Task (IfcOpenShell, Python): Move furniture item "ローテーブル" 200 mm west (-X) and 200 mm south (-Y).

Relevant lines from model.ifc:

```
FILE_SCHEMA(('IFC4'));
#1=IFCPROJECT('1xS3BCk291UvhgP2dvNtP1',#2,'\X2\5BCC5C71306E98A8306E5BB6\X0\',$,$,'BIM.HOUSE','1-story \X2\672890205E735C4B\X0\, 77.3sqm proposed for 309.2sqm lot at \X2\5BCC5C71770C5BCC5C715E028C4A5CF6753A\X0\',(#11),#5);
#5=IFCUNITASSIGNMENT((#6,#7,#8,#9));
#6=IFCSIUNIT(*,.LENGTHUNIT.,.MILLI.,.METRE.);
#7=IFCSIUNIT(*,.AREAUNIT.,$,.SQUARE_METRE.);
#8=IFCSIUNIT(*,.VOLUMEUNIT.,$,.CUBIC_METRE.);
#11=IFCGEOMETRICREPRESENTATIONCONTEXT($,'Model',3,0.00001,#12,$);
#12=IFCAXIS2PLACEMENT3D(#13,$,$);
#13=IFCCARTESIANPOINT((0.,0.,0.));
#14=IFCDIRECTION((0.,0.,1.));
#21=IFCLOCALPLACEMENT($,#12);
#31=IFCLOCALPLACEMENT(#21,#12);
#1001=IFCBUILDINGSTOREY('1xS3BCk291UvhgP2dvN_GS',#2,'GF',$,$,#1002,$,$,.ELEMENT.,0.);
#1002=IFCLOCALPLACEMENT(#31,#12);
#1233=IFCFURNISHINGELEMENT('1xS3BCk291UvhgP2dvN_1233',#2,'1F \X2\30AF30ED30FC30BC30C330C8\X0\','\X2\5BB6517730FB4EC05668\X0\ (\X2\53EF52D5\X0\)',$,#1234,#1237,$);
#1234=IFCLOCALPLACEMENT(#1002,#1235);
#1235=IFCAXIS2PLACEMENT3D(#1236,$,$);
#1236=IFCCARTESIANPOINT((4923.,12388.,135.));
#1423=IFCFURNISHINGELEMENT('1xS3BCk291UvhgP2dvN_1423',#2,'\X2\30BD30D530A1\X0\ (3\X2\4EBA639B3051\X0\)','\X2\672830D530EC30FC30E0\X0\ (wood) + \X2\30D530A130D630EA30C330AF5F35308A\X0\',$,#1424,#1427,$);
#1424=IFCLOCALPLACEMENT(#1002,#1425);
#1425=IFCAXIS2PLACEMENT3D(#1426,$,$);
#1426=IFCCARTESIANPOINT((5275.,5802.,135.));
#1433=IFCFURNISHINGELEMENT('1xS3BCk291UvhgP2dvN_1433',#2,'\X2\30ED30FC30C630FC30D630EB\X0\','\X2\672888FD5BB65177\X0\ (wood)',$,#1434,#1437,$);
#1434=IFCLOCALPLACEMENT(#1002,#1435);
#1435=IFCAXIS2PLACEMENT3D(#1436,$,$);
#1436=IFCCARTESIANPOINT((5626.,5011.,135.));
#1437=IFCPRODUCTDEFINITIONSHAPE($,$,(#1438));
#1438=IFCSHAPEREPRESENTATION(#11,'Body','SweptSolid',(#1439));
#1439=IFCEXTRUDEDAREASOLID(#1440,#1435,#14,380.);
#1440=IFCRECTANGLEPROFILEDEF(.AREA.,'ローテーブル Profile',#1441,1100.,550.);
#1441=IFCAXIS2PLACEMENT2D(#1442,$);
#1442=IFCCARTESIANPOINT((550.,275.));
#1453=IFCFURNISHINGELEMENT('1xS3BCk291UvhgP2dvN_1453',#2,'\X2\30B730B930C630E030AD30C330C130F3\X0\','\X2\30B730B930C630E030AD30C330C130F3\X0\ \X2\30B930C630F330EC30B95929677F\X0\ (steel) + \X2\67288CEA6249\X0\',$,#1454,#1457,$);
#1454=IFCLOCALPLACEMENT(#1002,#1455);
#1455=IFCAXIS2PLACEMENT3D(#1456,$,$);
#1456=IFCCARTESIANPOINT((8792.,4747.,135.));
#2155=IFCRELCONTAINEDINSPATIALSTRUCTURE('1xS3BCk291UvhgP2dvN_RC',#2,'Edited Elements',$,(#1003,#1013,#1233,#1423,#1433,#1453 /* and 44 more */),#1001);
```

```python
import ifcopenshell
import ifcopenshell.api.geometry
import ifcopenshell.util.placement
import ifcopenshell.util.unit

model = ifcopenshell.open("model.ifc")
unit_scale = ifcopenshell.util.unit.calculate_unit_scale(model)

item = model.by_guid("1xS3BCk291UvhgP2dvN_1433")
matrix = ifcopenshell.util.placement.get_local_placement(item.ObjectPlacement)
matrix[0, 3] -= 0.2 / unit_scale
matrix[1, 3] -= 0.2 / unit_scale
ifcopenshell.api.geometry.edit_object_placement(model, product=item, matrix=matrix, is_si=False)

print(ifcopenshell.util.placement.get_local_placement(item.ObjectPlacement).round(3) + 0.0)

model.write("model-out.ifc")
```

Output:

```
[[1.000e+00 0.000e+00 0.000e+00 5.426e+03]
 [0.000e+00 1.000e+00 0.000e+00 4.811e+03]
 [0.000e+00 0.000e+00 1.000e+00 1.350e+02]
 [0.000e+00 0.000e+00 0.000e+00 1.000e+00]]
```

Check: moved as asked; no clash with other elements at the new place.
